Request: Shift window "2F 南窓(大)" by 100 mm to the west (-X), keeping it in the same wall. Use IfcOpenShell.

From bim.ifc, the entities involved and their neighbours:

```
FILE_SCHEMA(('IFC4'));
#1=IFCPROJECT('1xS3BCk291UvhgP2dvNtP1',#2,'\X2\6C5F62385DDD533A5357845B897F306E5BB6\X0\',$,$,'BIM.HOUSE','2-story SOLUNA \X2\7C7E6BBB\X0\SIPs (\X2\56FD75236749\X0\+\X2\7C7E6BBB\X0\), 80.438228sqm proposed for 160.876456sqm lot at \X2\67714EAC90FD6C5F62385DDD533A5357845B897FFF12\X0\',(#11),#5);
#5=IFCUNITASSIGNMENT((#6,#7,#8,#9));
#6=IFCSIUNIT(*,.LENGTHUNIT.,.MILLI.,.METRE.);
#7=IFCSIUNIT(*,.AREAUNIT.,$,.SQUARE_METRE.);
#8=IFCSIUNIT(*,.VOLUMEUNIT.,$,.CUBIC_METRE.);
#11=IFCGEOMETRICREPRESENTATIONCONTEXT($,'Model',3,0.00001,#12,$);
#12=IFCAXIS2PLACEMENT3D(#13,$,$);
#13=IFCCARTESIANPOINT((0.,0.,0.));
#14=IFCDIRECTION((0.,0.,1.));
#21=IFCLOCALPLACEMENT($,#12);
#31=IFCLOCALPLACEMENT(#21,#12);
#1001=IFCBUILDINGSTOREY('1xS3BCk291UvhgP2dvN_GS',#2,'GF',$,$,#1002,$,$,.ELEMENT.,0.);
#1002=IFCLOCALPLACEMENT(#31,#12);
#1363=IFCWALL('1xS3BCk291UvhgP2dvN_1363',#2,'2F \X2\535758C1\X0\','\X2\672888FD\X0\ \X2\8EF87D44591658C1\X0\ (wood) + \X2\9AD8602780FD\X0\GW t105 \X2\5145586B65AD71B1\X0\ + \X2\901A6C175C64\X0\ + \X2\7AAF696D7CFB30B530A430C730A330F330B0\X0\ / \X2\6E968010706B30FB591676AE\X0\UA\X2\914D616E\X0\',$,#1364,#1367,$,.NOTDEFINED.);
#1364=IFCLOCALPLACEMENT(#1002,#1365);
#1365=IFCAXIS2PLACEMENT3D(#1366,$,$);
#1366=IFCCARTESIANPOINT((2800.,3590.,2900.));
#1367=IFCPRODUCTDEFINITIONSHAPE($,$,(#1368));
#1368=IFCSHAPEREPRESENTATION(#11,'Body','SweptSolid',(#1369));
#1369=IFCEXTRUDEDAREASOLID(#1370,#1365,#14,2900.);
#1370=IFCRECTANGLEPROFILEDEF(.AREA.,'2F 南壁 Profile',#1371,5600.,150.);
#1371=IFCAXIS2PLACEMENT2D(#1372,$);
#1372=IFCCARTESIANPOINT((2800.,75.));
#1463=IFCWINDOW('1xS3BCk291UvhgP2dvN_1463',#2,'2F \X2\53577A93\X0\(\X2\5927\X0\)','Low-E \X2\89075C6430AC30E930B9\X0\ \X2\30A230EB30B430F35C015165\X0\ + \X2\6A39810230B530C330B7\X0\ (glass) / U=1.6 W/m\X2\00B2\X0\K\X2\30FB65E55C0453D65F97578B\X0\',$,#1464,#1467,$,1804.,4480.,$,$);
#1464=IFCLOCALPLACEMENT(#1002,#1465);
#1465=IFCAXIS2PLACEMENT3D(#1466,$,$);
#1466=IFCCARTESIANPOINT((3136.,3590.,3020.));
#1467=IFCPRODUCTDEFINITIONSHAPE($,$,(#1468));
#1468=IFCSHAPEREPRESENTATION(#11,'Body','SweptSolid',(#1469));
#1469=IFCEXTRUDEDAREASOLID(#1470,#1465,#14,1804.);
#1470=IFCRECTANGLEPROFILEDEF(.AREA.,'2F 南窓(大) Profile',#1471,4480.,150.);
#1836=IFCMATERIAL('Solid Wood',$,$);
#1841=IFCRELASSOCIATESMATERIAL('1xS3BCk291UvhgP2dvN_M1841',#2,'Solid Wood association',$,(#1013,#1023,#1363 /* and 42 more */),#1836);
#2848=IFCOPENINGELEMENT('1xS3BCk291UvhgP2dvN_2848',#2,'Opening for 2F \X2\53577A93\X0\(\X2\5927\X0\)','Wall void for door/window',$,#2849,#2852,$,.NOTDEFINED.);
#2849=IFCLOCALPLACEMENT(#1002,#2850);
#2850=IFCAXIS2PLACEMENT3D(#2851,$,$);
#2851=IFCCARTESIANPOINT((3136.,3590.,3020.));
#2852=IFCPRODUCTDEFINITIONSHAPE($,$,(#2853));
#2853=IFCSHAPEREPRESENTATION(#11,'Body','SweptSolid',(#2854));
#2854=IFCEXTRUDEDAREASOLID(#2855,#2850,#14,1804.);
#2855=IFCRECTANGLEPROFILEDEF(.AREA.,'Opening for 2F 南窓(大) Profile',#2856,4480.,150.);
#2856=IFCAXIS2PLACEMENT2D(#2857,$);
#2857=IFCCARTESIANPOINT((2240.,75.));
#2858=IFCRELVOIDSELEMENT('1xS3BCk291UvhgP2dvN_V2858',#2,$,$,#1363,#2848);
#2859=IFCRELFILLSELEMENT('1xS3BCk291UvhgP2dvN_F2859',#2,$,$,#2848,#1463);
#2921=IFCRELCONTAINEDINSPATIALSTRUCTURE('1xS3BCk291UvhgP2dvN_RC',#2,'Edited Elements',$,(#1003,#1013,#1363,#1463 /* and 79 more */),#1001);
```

```python
import ifcopenshell
import ifcopenshell.api.geometry
import ifcopenshell.util.placement
import ifcopenshell.util.unit

model = ifcopenshell.open("bim.ifc")
unit_scale = ifcopenshell.util.unit.calculate_unit_scale(model)

window = model.by_guid("1xS3BCk291UvhgP2dvN_1463")
opening = window.FillsVoids[0].RelatingOpeningElement
wall = opening.VoidsElements[0].RelatingBuildingElement

wall_matrix = ifcopenshell.util.placement.get_local_placement(wall.ObjectPlacement)
shift = wall_matrix[:3, 0] * -0.1 / unit_scale
before = ifcopenshell.util.placement.get_local_placement(window.ObjectPlacement)[:3, 3].copy()

# The window is not placed relative to its opening, so move both.
for product in (opening, window):
    matrix = ifcopenshell.util.placement.get_local_placement(product.ObjectPlacement)
    matrix[:3, 3] += shift
    ifcopenshell.api.geometry.edit_object_placement(model, product=product, matrix=matrix, is_si=False)

after = ifcopenshell.util.placement.get_local_placement(window.ObjectPlacement)[:3, 3]
print("window moved by", (after - before).round(3) + 0.0)

model.write("bim_rev.ifc")
```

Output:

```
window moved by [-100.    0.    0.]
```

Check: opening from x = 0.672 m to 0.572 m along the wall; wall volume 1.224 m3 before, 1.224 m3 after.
